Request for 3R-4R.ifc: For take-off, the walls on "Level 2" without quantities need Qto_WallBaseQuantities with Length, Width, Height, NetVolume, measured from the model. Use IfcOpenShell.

First a look at what the model holds.

```python
import ifcopenshell
import ifcopenshell.util.element
import ifcopenshell.util.unit

model = ifcopenshell.open("3R-4R.ifc")
print(model.schema)
for unit_type in ("LENGTHUNIT", "AREAUNIT", "VOLUMEUNIT"):
    print(unit_type, ifcopenshell.util.unit.calculate_unit_scale(model, unit_type))
storey = next(s for s in model.by_type("IfcBuildingStorey") if s.Name == "Level 2")
walls = [e for e in ifcopenshell.util.element.get_decomposition(storey) if e.is_a("IfcWall")]
for e in sorted(walls, key=lambda e: e.id()):
    print(e.id(), e.is_a(), e.Name, list(ifcopenshell.util.element.get_psets(e, qtos_only=True)), sep=" | ")
```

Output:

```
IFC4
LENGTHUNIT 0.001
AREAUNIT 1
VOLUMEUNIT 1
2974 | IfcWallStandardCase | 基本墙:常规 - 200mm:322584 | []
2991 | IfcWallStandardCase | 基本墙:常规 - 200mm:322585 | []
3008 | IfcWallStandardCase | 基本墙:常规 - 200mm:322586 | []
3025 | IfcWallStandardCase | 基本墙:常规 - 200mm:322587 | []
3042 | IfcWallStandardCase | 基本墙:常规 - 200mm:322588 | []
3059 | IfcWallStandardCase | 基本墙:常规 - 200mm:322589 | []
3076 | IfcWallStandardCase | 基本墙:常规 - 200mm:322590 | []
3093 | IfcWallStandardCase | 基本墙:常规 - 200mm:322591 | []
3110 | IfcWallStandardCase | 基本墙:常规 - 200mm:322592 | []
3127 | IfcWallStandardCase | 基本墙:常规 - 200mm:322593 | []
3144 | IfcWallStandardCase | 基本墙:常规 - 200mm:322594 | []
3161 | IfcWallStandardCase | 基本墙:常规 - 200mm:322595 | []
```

```python
import ifcopenshell
import ifcopenshell.api.pset
import ifcopenshell.geom
import ifcopenshell.util.element
import ifcopenshell.util.shape
import ifcopenshell.util.unit

model = ifcopenshell.open("3R-4R.ifc")
unit_scale = ifcopenshell.util.unit.calculate_unit_scale(model)
volume_scale = ifcopenshell.util.unit.calculate_unit_scale(model, "VOLUMEUNIT")
settings = ifcopenshell.geom.settings()

storey = next(s for s in model.by_type("IfcBuildingStorey") if s.Name == "Level 2")
walls = [e for e in ifcopenshell.util.element.get_decomposition(storey) if e.is_a("IfcWall")]

for e in sorted(walls, key=lambda e: e.id()):
    if ifcopenshell.util.element.get_psets(e, qtos_only=True, should_inherit=False):
        continue
    # Geometry comes back in metres, in the element's own axes.
    shape = ifcopenshell.geom.create_shape(settings, e)
    values = {
        "Length": ifcopenshell.util.shape.get_x(shape.geometry) / unit_scale,
        "Width": ifcopenshell.util.shape.get_y(shape.geometry) / unit_scale,
        "Height": ifcopenshell.util.shape.get_z(shape.geometry) / unit_scale,
        "NetVolume": ifcopenshell.util.shape.get_volume(shape.geometry) / volume_scale,
    }
    qto = ifcopenshell.api.pset.add_qto(model, product=e, name="Qto_WallBaseQuantities")
    ifcopenshell.api.pset.edit_qto(model, qto=qto, properties=values)
    print(e.id(), {k: round(v, 3) for k, v in values.items()})

model.write("3R-4R-out.ifc")
```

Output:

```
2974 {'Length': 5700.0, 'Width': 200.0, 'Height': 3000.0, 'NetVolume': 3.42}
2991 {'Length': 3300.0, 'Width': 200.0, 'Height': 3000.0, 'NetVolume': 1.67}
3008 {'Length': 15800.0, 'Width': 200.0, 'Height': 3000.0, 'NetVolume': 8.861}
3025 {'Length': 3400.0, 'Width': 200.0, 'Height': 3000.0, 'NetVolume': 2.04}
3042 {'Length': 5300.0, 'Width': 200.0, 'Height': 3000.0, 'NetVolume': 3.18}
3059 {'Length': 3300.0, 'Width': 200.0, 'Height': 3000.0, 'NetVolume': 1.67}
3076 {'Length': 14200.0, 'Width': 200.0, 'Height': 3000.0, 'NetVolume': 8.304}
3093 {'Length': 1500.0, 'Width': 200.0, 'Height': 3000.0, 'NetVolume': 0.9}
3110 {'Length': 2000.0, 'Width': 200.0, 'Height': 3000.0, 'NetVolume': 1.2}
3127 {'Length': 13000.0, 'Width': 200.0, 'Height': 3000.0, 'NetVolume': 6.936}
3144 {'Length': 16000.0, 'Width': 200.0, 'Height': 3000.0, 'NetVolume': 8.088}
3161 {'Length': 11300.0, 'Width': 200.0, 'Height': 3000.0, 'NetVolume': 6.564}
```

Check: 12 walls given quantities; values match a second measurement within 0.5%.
